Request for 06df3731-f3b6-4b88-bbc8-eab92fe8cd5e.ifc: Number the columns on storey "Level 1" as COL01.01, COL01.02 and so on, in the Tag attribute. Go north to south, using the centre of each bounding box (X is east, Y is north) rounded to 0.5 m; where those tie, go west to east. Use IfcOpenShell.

First a look at what the model holds.

```python
import ifcopenshell
import ifcopenshell.util.element
import ifcopenshell.util.placement

model = ifcopenshell.open("06df3731-f3b6-4b88-bbc8-eab92fe8cd5e.ifc")
print(model.schema)
storey = next(s for s in model.by_type("IfcBuildingStorey") if s.Name == "Level 1")
columns = [e for e in ifcopenshell.util.element.get_decomposition(storey) if e.is_a("IfcColumn")]
for e in sorted(columns, key=lambda e: e.id()):
    origin = ifcopenshell.util.placement.get_local_placement(e.ObjectPlacement)[:3, 3]
    print(e.id(), e.Tag, e.Name, origin.round(2) + 0.0, sep=" | ")
```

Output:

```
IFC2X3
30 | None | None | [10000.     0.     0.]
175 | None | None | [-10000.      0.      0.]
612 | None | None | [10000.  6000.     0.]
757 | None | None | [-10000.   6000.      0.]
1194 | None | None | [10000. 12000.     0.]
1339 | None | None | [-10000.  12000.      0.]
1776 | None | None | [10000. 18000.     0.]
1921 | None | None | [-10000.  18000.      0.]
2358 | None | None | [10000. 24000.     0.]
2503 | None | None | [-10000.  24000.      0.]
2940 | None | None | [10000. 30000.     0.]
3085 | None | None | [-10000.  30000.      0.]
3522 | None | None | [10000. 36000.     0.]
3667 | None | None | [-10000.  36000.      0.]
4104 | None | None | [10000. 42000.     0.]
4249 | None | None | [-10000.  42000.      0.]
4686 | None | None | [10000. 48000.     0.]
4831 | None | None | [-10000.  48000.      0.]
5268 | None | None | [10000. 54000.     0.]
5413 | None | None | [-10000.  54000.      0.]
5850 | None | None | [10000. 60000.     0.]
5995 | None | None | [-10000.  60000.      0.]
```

```python
import ifcopenshell
import ifcopenshell.geom
import ifcopenshell.util.element
import ifcopenshell.util.shape

model = ifcopenshell.open("06df3731-f3b6-4b88-bbc8-eab92fe8cd5e.ifc")
settings = ifcopenshell.geom.settings()
settings.set("use-world-coords", True)


def centre(element):
    shape = ifcopenshell.geom.create_shape(settings, element)
    return ifcopenshell.util.shape.get_bbox_centroid(shape.geometry)


storey = next(s for s in model.by_type("IfcBuildingStorey") if s.Name == "Level 1")
columns = [e for e in ifcopenshell.util.element.get_decomposition(storey) if e.is_a("IfcColumn")]

# Insertion points can sit at a corner or the storey origin, so sort by the geometry (in metres).
centres = {e: centre(e) for e in columns}
columns.sort(key=lambda e: (-round(centres[e][1] / 0.5), centres[e][0]))

for i, e in enumerate(columns, start=1):
    number = f"COL01.{i:02d}"
    e.Tag = number
    print(e.id(), number)

model.write("06df3731-f3b6-4b88-bbc8-eab92fe8cd5e-out.ifc")
```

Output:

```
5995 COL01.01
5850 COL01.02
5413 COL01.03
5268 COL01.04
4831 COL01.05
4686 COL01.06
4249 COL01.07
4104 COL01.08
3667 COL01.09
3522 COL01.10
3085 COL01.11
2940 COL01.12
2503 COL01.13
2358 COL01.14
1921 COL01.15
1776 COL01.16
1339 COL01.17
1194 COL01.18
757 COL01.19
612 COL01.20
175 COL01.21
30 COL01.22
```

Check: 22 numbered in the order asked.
